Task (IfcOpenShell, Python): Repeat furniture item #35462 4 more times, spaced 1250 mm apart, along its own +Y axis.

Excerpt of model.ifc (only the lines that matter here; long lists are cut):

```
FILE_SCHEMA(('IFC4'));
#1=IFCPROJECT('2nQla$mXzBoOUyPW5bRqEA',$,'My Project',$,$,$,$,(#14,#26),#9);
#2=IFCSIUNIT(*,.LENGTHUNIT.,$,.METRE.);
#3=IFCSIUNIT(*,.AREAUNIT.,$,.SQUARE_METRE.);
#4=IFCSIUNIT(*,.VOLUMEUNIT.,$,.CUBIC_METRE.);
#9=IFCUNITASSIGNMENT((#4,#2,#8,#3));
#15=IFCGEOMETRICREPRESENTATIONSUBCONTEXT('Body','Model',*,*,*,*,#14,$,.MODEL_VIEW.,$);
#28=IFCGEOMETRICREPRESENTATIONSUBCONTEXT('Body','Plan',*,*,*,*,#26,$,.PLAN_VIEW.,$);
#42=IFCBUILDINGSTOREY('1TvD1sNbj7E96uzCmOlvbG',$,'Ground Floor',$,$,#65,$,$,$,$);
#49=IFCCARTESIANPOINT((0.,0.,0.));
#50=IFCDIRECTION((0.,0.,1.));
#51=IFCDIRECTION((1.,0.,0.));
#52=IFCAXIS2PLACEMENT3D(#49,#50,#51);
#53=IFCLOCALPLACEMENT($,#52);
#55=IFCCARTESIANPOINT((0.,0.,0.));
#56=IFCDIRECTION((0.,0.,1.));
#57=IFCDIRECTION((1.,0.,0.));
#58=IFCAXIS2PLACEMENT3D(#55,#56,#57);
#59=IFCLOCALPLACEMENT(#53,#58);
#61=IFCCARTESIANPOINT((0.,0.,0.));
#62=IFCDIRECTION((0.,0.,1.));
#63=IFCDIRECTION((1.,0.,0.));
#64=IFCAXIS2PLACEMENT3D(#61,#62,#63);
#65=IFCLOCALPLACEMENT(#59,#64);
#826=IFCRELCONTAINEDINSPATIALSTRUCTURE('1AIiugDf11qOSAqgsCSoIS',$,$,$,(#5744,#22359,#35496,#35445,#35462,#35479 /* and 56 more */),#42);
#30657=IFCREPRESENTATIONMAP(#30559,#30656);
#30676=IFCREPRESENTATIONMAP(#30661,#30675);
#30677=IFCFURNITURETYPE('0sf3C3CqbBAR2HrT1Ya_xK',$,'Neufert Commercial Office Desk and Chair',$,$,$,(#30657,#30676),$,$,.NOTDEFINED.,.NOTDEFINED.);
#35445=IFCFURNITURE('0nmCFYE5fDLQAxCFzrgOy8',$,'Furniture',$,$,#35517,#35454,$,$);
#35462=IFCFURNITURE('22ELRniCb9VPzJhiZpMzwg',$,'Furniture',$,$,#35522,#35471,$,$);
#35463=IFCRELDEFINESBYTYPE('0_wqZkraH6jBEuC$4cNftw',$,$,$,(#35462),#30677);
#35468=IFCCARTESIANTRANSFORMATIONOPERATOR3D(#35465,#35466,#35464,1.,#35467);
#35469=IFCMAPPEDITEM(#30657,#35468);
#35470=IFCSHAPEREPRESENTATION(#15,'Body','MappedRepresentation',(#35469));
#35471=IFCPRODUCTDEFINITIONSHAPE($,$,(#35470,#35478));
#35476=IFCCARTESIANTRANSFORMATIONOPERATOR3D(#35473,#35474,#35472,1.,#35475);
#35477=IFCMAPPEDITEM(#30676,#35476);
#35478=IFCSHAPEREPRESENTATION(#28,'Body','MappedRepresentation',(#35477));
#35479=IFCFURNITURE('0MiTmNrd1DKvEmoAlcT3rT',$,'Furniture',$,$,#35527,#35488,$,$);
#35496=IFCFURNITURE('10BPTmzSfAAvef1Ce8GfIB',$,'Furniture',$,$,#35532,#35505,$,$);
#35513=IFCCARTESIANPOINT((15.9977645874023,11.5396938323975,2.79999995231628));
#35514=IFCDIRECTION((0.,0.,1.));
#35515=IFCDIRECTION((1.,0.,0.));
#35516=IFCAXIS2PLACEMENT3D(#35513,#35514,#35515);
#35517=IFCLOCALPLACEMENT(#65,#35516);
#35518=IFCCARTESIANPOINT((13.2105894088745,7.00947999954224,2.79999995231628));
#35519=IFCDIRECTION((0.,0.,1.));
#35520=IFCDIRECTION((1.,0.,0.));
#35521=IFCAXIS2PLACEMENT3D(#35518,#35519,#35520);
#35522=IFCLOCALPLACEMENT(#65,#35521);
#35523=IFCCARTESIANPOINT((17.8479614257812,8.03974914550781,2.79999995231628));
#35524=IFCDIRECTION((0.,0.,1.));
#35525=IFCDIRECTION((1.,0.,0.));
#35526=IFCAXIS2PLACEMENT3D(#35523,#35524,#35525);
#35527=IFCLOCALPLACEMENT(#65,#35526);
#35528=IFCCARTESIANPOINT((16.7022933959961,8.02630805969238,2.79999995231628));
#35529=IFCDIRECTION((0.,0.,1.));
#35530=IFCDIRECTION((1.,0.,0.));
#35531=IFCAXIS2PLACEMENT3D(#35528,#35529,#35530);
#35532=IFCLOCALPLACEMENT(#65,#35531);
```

```python
import ifcopenshell
import ifcopenshell.api.geometry
import ifcopenshell.api.root
import ifcopenshell.util.element
import ifcopenshell.util.placement
import ifcopenshell.util.unit

model = ifcopenshell.open("model.ifc")
unit_scale = ifcopenshell.util.unit.calculate_unit_scale(model)

source = model.by_guid("22ELRniCb9VPzJhiZpMzwg")
base = ifcopenshell.util.placement.get_local_placement(source.ObjectPlacement)
step = base[:3, 1] * 1.25 / unit_scale

for i in range(1, 5):
    copy = ifcopenshell.api.root.copy_class(model, product=source)
    copy.Representation = ifcopenshell.util.element.copy_deep(
        model, source.Representation, exclude=["IfcGeometricRepresentationContext", "IfcRepresentationMap"]
    )
    matrix = base.copy()
    matrix[:3, 3] += i * step
    print("added at", matrix[:3, 3].round(3) + 0.0)
    ifcopenshell.api.geometry.edit_object_placement(model, product=copy, matrix=matrix, is_si=False)

model.write("model_edited.ifc")
```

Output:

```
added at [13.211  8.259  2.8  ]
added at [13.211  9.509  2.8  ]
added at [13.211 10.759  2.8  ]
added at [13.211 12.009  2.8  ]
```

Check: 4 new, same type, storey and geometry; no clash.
